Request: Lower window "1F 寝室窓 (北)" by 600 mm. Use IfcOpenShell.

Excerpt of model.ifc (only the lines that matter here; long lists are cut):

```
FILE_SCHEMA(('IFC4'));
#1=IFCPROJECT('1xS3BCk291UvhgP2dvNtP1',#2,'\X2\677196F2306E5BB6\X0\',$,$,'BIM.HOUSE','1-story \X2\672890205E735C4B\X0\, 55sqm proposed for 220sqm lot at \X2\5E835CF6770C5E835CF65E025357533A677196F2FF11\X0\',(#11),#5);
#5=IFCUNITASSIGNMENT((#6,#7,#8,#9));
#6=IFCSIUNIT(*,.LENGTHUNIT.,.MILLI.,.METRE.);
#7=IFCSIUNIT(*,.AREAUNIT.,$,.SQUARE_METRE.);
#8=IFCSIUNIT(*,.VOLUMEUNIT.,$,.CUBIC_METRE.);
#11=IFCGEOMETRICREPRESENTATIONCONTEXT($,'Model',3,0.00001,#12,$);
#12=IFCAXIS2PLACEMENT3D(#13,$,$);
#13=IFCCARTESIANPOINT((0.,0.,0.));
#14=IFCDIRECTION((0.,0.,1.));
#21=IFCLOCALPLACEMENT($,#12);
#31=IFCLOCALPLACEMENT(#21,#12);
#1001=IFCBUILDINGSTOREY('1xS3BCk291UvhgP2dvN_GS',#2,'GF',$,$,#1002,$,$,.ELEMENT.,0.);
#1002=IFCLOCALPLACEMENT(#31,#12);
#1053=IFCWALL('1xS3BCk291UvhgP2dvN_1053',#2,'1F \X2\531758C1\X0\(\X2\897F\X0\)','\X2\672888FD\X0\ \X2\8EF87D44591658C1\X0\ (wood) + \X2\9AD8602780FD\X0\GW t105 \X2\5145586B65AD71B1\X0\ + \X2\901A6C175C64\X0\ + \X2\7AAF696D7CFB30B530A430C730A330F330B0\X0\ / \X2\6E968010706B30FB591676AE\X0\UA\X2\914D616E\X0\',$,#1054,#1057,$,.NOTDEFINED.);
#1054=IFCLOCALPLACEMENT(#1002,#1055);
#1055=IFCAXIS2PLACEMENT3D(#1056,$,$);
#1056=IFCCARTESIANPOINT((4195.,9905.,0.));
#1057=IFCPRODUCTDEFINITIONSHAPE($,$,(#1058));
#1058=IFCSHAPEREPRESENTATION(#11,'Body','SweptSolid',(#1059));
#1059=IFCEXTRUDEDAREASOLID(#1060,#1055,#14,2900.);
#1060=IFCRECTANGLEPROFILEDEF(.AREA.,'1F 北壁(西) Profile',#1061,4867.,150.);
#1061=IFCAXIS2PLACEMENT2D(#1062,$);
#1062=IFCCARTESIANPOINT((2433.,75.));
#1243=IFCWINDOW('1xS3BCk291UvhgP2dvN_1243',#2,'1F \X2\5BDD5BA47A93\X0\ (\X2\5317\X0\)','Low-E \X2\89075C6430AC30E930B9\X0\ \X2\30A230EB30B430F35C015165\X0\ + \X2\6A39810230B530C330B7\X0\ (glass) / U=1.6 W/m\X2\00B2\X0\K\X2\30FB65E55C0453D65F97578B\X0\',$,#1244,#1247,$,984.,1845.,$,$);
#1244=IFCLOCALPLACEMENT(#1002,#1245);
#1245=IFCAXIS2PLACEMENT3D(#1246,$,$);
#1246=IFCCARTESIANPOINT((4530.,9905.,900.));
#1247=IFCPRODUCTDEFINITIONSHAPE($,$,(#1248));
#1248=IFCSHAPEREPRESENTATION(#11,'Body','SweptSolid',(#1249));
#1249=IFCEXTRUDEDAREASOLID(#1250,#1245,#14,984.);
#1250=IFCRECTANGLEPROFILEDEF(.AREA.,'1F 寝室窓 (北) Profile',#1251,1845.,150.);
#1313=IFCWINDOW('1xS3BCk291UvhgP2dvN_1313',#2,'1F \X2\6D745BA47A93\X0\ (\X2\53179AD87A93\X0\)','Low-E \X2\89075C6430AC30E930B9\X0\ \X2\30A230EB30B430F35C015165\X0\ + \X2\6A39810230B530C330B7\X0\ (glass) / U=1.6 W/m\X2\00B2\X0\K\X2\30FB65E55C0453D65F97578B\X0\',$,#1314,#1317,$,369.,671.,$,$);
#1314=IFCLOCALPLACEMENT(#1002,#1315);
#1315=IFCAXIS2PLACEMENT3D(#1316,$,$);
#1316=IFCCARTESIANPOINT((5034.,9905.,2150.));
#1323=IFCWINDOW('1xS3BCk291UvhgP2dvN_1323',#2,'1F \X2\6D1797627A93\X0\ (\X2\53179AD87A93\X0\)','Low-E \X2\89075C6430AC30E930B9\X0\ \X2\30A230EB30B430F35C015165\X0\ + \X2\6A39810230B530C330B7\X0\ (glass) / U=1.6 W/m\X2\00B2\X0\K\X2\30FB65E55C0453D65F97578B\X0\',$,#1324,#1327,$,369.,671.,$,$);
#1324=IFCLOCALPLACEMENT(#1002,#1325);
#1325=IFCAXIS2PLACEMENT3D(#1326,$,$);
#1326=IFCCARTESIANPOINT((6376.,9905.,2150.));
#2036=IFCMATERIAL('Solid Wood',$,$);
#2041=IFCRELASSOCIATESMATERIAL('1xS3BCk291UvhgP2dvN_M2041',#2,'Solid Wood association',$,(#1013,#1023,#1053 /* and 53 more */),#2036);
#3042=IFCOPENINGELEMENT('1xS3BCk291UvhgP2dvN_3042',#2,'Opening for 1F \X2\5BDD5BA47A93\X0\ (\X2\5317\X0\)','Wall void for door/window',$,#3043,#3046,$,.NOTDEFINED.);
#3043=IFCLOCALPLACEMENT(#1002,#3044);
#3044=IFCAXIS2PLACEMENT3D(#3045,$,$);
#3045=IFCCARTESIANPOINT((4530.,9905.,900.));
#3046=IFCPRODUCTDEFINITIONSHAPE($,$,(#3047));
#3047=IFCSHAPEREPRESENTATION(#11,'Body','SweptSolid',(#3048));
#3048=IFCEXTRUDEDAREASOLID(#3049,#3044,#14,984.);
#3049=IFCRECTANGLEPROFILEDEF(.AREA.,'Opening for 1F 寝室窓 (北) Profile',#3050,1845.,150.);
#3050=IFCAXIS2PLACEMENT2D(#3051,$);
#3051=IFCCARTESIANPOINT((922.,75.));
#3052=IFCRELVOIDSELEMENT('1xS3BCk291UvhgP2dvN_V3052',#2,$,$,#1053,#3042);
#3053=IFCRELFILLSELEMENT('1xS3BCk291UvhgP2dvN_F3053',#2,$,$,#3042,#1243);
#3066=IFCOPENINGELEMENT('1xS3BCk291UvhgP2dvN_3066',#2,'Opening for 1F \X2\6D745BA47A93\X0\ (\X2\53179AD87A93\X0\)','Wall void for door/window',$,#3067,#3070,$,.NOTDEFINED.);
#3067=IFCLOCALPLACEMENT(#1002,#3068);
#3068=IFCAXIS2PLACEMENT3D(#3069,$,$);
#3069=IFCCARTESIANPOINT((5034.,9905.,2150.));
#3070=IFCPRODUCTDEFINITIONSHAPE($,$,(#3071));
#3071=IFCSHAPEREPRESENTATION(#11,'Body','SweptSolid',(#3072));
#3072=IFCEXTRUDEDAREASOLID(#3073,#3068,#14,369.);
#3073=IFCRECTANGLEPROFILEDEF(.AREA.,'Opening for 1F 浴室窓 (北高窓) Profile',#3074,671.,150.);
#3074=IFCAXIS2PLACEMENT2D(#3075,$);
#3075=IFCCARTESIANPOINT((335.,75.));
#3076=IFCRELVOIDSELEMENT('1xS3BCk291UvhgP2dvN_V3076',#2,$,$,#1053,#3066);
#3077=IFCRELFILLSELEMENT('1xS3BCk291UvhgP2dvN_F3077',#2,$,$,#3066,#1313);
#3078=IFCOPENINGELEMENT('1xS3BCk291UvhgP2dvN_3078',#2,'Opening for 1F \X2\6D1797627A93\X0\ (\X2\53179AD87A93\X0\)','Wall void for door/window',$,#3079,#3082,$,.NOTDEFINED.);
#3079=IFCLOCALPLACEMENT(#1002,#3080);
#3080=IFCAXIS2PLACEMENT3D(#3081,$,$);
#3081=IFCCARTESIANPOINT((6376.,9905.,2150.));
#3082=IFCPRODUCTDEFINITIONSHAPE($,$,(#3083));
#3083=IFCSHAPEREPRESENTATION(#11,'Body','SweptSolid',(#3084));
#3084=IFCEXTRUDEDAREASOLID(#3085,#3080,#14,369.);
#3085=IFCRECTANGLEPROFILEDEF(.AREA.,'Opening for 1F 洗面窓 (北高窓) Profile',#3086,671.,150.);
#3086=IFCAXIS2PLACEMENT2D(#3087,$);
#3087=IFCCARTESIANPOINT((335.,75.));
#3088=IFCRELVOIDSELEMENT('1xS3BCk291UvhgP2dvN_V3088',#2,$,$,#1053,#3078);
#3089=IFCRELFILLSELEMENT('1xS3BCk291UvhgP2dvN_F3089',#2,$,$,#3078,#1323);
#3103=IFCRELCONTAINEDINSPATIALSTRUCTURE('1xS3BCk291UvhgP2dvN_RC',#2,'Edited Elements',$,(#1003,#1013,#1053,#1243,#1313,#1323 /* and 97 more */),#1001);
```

```python
import numpy as np
import ifcopenshell
import ifcopenshell.api.geometry
import ifcopenshell.util.placement
import ifcopenshell.util.unit

model = ifcopenshell.open("model.ifc")
unit_scale = ifcopenshell.util.unit.calculate_unit_scale(model)

window = model.by_guid("1xS3BCk291UvhgP2dvN_1243")
opening = window.FillsVoids[0].RelatingOpeningElement
dz = -0.6 / unit_scale

shift = np.array([0.0, 0.0, dz])
# The window is not placed relative to its opening, so move both.
for product in (opening, window):
    matrix = ifcopenshell.util.placement.get_local_placement(product.ObjectPlacement)
    matrix[:3, 3] += shift
    ifcopenshell.api.geometry.edit_object_placement(model, product=product, matrix=matrix, is_si=False)

print(f"moved by {dz * unit_scale:+.3f} m")

model.write("model_v2.ifc")
```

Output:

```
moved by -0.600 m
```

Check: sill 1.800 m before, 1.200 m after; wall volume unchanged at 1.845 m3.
